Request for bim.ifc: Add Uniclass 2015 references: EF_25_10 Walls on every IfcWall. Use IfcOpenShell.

First a look at what the model holds.

```python
import ifcopenshell

model = ifcopenshell.open("bim.ifc")
print(model.schema)
print("classifications:", [c.Name for c in model.by_type("IfcClassification")])
for ifc_class in ("IfcDoor", "IfcRoof", "IfcStair", "IfcWall", "IfcWindow"):
    print(ifc_class, len(model.by_type(ifc_class)))
```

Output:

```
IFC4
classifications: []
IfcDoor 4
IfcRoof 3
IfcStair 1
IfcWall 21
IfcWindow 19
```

```python
import ifcopenshell
import ifcopenshell.api.classification

model = ifcopenshell.open("bim.ifc")

system = ifcopenshell.api.classification.add_classification(model, classification="Uniclass 2015")

codes = {
    "IfcWall": ("EF_25_10", "Walls"),
}
for ifc_class, (code, name) in codes.items():
    products = model.by_type(ifc_class)
    ifcopenshell.api.classification.add_reference(
        model, products=products, classification=system, identification=code, name=name
    )
    print(code, len(products))

model.write("bim_edited.ifc")
```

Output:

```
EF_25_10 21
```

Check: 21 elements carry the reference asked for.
